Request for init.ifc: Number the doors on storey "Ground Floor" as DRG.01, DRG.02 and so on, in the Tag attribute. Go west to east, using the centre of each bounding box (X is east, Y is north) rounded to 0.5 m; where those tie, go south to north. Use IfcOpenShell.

First a look at what the model holds.

```python
import ifcopenshell
import ifcopenshell.util.element
import ifcopenshell.util.placement

model = ifcopenshell.open("init.ifc")
print(model.schema)
storey = next(s for s in model.by_type("IfcBuildingStorey") if s.Name == "Ground Floor")
doors = [e for e in ifcopenshell.util.element.get_decomposition(storey) if e.is_a("IfcDoor")]
for e in sorted(doors, key=lambda e: e.id()):
    origin = ifcopenshell.util.placement.get_local_placement(e.ObjectPlacement)[:3, 3]
    print(e.id(), e.Tag, e.Name, origin.round(2) + 0.0, sep=" | ")
```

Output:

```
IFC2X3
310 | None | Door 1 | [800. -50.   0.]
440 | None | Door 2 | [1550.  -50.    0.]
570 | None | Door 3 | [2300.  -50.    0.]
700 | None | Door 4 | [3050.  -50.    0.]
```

```python
import ifcopenshell
import ifcopenshell.geom
import ifcopenshell.util.element
import ifcopenshell.util.shape

model = ifcopenshell.open("init.ifc")
settings = ifcopenshell.geom.settings()
settings.set("use-world-coords", True)


def centre(element):
    shape = ifcopenshell.geom.create_shape(settings, element)
    return ifcopenshell.util.shape.get_bbox_centroid(shape.geometry)


storey = next(s for s in model.by_type("IfcBuildingStorey") if s.Name == "Ground Floor")
doors = [e for e in ifcopenshell.util.element.get_decomposition(storey) if e.is_a("IfcDoor")]

# Insertion points can sit at a corner or the storey origin, so sort by the geometry (in metres).
centres = {e: centre(e) for e in doors}
doors.sort(key=lambda e: (round(centres[e][0] / 0.5), centres[e][1]))

for i, e in enumerate(doors, start=1):
    number = f"DRG.{i:02d}"
    e.Tag = number
    print(e.id(), number)

model.write("init_edited.ifc")
```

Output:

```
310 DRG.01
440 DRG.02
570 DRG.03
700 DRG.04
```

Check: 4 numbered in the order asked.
